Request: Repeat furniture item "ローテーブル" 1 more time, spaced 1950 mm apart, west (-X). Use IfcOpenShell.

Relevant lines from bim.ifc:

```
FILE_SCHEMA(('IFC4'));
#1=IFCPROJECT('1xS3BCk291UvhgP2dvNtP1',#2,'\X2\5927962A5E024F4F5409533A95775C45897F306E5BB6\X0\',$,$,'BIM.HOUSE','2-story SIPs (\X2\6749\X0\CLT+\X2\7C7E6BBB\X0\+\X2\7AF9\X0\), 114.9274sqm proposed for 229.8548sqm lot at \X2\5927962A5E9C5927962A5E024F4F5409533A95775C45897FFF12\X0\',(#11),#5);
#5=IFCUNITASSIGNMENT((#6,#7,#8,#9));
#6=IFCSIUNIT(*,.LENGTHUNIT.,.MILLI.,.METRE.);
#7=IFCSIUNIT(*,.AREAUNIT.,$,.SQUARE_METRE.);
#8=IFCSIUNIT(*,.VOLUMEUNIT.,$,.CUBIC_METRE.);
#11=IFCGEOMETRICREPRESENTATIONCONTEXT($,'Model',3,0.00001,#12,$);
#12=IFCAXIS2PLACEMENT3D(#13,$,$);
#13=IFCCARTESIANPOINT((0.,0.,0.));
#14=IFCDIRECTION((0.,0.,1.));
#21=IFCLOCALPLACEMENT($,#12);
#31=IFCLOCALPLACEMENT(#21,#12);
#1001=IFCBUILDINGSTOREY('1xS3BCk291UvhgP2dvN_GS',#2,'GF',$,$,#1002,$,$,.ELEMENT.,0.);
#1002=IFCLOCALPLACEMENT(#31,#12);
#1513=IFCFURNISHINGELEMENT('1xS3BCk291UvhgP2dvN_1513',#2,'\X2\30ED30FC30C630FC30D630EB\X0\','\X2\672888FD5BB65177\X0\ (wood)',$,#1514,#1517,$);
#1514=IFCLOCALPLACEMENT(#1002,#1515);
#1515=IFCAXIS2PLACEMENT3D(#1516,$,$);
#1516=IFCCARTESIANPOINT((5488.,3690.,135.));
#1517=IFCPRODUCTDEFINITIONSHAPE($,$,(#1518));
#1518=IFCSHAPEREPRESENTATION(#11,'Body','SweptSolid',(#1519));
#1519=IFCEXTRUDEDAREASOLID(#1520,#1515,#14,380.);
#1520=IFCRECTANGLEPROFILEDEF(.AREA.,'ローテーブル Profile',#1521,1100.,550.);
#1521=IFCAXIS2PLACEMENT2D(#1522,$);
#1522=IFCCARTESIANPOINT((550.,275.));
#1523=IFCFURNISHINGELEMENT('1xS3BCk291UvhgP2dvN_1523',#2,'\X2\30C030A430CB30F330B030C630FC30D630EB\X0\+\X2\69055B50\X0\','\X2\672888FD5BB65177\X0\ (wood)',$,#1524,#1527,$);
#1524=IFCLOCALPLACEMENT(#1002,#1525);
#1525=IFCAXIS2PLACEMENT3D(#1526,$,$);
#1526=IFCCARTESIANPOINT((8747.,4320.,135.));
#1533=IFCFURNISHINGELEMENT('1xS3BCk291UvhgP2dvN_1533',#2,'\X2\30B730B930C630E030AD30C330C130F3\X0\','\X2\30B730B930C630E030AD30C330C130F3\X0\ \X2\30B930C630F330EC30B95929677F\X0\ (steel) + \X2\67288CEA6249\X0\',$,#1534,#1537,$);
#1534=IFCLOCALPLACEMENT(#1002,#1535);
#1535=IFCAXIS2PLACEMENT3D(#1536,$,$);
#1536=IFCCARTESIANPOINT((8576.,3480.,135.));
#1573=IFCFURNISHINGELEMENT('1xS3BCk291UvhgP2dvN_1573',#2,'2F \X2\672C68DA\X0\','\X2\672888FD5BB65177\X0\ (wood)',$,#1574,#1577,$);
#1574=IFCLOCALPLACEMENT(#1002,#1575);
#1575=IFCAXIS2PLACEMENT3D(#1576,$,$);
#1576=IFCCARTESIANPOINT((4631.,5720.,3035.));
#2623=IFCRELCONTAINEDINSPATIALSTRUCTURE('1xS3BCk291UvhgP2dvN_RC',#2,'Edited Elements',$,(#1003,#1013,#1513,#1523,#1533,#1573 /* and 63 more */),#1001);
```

```python
import numpy as np
import ifcopenshell
import ifcopenshell.api.geometry
import ifcopenshell.api.root
import ifcopenshell.util.element
import ifcopenshell.util.placement
import ifcopenshell.util.unit

model = ifcopenshell.open("bim.ifc")
unit_scale = ifcopenshell.util.unit.calculate_unit_scale(model)


def reuse_history(source, copy):
    """copy_class also copies each property set's owner history, people and application; keep the originals."""
    for rel in copy.IsDefinedBy:
        if rel.is_a("IfcRelDefinesByProperties") and (history := rel.RelatingPropertyDefinition.OwnerHistory):
            rel.RelatingPropertyDefinition.OwnerHistory = source.OwnerHistory
            ifcopenshell.util.element.remove_deep2(model, history)


source = model.by_guid("1xS3BCk291UvhgP2dvN_1513")
base = ifcopenshell.util.placement.get_local_placement(source.ObjectPlacement)
step = np.array([-1.0, 0.0, 0.0]) * 1.95 / unit_scale

for i in range(1, 2):
    copy = ifcopenshell.api.root.copy_class(model, product=source)
    copy.Representation = ifcopenshell.util.element.copy_deep(
        model, source.Representation, exclude=["IfcGeometricRepresentationContext", "IfcRepresentationMap"]
    )
    reuse_history(source, copy)
    matrix = base.copy()
    matrix[:3, 3] += i * step
    print("added at", matrix[:3, 3].round(3) + 0.0)
    ifcopenshell.api.geometry.edit_object_placement(model, product=copy, matrix=matrix, is_si=False)

model.write("bim_rev.ifc")
```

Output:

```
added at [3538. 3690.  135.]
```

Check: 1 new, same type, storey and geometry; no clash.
